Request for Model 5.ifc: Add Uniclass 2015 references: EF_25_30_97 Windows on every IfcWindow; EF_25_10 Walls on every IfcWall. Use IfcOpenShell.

First a look at what the model holds.

```python
import ifcopenshell

model = ifcopenshell.open("Model 5.ifc")
print(model.schema)
print("classifications:", [c.Name for c in model.by_type("IfcClassification")])
for ifc_class in ("IfcDoor", "IfcRoof", "IfcStair", "IfcWall", "IfcWindow"):
    print(ifc_class, len(model.by_type(ifc_class)))
```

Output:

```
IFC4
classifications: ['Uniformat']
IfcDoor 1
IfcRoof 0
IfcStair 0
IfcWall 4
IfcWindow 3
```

```python
import ifcopenshell
import ifcopenshell.api.classification

model = ifcopenshell.open("Model 5.ifc")

system = ifcopenshell.api.classification.add_classification(model, classification="Uniclass 2015")

codes = {
    "IfcWindow": ("EF_25_30_97", "Windows"),
    "IfcWall": ("EF_25_10", "Walls"),
}
for ifc_class, (code, name) in codes.items():
    products = model.by_type(ifc_class)
    ifcopenshell.api.classification.add_reference(
        model, products=products, classification=system, identification=code, name=name
    )
    print(code, len(products))

model.write("Model 5-out.ifc")
```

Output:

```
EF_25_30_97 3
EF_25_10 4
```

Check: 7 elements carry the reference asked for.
